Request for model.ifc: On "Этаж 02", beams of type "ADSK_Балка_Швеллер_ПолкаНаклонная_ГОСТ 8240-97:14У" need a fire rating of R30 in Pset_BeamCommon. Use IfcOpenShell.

First a look at what the model holds.

```python
import ifcopenshell
import ifcopenshell.util.element

model = ifcopenshell.open("model.ifc")
print(model.schema)
storey = next(s for s in model.by_type("IfcBuildingStorey") if s.Name == "Этаж 02")
beams = [e for e in ifcopenshell.util.element.get_decomposition(storey) if e.is_a("IfcBeam")]
seen = {}
for e in beams:
    element_type = ifcopenshell.util.element.get_type(e)
    key = (element_type.Name if element_type != e and element_type else None, ifcopenshell.util.element.get_pset(e, "Pset_BeamCommon", "FireRating"))
    seen[key] = seen.get(key, 0) + 1
for (name, value), count in sorted(seen.items(), key=str):
    print(count, "x", name, "|", value)
```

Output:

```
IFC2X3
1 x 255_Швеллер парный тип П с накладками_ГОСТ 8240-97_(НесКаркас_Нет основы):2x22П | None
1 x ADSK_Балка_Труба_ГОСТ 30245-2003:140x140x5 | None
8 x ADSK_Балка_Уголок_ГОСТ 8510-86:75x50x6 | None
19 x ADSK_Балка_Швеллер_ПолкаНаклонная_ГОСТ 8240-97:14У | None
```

```python
import ifcopenshell
import ifcopenshell.api.pset
import ifcopenshell.util.element

model = ifcopenshell.open("model.ifc")

storey = next(s for s in model.by_type("IfcBuildingStorey") if s.Name == "Этаж 02")
beams = [e for e in ifcopenshell.util.element.get_decomposition(storey) if e.is_a("IfcBeam")]

count = 0
for e in beams:
    element_type = ifcopenshell.util.element.get_type(e)
    if element_type in (None, e) or element_type.Name != "ADSK_Балка_Швеллер_ПолкаНаклонная_ГОСТ 8240-97:14У":
        continue
    # add_pset returns the element's existing set when there is one.
    pset = ifcopenshell.api.pset.add_pset(model, product=e, name="Pset_BeamCommon")
    ifcopenshell.api.pset.edit_pset(model, pset=pset, properties={"FireRating": "R30"})
    count += 1

print(count, "beams updated")

model.write("model_rev.ifc")
```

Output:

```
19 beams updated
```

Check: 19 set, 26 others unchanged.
